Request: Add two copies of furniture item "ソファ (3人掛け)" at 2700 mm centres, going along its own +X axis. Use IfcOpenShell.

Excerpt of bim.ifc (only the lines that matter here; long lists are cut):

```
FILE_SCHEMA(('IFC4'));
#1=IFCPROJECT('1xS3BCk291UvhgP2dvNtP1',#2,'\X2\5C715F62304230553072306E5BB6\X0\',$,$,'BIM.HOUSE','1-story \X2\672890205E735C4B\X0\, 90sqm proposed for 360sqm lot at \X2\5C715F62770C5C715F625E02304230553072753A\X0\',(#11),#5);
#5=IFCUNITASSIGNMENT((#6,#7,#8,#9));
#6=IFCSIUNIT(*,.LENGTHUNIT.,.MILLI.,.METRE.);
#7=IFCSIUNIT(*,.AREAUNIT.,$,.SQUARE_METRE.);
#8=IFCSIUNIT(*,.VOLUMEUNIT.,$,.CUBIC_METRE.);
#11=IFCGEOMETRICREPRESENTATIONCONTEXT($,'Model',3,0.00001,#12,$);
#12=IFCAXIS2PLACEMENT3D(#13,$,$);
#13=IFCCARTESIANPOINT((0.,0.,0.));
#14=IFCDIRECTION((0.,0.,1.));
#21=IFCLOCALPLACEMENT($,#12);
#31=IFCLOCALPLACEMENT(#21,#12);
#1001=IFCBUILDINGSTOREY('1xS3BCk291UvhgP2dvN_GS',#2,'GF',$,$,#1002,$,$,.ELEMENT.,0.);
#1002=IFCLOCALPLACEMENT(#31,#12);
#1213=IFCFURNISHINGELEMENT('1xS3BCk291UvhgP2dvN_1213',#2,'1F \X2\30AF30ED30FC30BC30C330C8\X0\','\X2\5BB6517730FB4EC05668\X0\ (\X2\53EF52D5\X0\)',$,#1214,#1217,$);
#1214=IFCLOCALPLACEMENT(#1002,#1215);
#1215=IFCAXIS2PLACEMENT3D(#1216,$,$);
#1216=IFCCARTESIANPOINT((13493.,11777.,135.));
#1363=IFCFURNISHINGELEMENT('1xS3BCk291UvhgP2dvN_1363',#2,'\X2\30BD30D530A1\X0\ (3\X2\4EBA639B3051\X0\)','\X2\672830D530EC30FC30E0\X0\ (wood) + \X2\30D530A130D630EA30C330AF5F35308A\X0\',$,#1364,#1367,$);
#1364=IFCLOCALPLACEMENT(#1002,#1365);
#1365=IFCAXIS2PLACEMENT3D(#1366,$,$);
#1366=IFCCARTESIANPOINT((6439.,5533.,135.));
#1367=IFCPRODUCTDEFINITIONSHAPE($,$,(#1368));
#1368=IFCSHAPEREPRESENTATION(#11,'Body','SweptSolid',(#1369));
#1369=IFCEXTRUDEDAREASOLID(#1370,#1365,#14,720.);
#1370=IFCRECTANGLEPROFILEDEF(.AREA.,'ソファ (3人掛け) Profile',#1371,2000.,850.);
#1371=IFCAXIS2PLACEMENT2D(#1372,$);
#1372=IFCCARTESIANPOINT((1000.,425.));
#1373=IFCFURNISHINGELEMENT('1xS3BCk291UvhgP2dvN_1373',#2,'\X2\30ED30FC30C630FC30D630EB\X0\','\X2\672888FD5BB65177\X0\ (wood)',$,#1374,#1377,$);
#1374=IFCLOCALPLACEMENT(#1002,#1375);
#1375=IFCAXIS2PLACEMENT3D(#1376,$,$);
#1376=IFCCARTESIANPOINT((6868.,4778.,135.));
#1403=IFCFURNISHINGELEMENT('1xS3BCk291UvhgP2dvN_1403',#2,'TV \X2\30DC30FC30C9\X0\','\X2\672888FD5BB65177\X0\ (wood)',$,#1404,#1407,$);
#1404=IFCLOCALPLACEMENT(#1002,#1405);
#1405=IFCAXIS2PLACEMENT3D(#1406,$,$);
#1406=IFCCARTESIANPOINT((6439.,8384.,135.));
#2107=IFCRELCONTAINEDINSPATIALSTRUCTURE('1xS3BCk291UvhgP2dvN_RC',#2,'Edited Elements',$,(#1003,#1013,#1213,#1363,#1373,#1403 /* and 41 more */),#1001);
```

```python
import ifcopenshell
import ifcopenshell.api.geometry
import ifcopenshell.api.root
import ifcopenshell.util.element
import ifcopenshell.util.placement
import ifcopenshell.util.unit

model = ifcopenshell.open("bim.ifc")
unit_scale = ifcopenshell.util.unit.calculate_unit_scale(model)


def reuse_history(source, copy):
    """copy_class also copies each property set's owner history, people and application; keep the originals."""
    for rel in copy.IsDefinedBy:
        if rel.is_a("IfcRelDefinesByProperties") and (history := rel.RelatingPropertyDefinition.OwnerHistory):
            rel.RelatingPropertyDefinition.OwnerHistory = source.OwnerHistory
            ifcopenshell.util.element.remove_deep2(model, history)


source = model.by_id(1363)
base = ifcopenshell.util.placement.get_local_placement(source.ObjectPlacement)
step = base[:3, 0] * 2.7 / unit_scale

for i in range(1, 3):
    copy = ifcopenshell.api.root.copy_class(model, product=source)
    copy.Representation = ifcopenshell.util.element.copy_deep(
        model, source.Representation, exclude=["IfcGeometricRepresentationContext", "IfcRepresentationMap"]
    )
    reuse_history(source, copy)
    matrix = base.copy()
    matrix[:3, 3] += i * step
    print("added at", matrix[:3, 3].round(3) + 0.0)
    ifcopenshell.api.geometry.edit_object_placement(model, product=copy, matrix=matrix, is_si=False)

model.write("bim_rev.ifc")
```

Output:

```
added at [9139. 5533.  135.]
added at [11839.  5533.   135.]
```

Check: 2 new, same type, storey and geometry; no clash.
